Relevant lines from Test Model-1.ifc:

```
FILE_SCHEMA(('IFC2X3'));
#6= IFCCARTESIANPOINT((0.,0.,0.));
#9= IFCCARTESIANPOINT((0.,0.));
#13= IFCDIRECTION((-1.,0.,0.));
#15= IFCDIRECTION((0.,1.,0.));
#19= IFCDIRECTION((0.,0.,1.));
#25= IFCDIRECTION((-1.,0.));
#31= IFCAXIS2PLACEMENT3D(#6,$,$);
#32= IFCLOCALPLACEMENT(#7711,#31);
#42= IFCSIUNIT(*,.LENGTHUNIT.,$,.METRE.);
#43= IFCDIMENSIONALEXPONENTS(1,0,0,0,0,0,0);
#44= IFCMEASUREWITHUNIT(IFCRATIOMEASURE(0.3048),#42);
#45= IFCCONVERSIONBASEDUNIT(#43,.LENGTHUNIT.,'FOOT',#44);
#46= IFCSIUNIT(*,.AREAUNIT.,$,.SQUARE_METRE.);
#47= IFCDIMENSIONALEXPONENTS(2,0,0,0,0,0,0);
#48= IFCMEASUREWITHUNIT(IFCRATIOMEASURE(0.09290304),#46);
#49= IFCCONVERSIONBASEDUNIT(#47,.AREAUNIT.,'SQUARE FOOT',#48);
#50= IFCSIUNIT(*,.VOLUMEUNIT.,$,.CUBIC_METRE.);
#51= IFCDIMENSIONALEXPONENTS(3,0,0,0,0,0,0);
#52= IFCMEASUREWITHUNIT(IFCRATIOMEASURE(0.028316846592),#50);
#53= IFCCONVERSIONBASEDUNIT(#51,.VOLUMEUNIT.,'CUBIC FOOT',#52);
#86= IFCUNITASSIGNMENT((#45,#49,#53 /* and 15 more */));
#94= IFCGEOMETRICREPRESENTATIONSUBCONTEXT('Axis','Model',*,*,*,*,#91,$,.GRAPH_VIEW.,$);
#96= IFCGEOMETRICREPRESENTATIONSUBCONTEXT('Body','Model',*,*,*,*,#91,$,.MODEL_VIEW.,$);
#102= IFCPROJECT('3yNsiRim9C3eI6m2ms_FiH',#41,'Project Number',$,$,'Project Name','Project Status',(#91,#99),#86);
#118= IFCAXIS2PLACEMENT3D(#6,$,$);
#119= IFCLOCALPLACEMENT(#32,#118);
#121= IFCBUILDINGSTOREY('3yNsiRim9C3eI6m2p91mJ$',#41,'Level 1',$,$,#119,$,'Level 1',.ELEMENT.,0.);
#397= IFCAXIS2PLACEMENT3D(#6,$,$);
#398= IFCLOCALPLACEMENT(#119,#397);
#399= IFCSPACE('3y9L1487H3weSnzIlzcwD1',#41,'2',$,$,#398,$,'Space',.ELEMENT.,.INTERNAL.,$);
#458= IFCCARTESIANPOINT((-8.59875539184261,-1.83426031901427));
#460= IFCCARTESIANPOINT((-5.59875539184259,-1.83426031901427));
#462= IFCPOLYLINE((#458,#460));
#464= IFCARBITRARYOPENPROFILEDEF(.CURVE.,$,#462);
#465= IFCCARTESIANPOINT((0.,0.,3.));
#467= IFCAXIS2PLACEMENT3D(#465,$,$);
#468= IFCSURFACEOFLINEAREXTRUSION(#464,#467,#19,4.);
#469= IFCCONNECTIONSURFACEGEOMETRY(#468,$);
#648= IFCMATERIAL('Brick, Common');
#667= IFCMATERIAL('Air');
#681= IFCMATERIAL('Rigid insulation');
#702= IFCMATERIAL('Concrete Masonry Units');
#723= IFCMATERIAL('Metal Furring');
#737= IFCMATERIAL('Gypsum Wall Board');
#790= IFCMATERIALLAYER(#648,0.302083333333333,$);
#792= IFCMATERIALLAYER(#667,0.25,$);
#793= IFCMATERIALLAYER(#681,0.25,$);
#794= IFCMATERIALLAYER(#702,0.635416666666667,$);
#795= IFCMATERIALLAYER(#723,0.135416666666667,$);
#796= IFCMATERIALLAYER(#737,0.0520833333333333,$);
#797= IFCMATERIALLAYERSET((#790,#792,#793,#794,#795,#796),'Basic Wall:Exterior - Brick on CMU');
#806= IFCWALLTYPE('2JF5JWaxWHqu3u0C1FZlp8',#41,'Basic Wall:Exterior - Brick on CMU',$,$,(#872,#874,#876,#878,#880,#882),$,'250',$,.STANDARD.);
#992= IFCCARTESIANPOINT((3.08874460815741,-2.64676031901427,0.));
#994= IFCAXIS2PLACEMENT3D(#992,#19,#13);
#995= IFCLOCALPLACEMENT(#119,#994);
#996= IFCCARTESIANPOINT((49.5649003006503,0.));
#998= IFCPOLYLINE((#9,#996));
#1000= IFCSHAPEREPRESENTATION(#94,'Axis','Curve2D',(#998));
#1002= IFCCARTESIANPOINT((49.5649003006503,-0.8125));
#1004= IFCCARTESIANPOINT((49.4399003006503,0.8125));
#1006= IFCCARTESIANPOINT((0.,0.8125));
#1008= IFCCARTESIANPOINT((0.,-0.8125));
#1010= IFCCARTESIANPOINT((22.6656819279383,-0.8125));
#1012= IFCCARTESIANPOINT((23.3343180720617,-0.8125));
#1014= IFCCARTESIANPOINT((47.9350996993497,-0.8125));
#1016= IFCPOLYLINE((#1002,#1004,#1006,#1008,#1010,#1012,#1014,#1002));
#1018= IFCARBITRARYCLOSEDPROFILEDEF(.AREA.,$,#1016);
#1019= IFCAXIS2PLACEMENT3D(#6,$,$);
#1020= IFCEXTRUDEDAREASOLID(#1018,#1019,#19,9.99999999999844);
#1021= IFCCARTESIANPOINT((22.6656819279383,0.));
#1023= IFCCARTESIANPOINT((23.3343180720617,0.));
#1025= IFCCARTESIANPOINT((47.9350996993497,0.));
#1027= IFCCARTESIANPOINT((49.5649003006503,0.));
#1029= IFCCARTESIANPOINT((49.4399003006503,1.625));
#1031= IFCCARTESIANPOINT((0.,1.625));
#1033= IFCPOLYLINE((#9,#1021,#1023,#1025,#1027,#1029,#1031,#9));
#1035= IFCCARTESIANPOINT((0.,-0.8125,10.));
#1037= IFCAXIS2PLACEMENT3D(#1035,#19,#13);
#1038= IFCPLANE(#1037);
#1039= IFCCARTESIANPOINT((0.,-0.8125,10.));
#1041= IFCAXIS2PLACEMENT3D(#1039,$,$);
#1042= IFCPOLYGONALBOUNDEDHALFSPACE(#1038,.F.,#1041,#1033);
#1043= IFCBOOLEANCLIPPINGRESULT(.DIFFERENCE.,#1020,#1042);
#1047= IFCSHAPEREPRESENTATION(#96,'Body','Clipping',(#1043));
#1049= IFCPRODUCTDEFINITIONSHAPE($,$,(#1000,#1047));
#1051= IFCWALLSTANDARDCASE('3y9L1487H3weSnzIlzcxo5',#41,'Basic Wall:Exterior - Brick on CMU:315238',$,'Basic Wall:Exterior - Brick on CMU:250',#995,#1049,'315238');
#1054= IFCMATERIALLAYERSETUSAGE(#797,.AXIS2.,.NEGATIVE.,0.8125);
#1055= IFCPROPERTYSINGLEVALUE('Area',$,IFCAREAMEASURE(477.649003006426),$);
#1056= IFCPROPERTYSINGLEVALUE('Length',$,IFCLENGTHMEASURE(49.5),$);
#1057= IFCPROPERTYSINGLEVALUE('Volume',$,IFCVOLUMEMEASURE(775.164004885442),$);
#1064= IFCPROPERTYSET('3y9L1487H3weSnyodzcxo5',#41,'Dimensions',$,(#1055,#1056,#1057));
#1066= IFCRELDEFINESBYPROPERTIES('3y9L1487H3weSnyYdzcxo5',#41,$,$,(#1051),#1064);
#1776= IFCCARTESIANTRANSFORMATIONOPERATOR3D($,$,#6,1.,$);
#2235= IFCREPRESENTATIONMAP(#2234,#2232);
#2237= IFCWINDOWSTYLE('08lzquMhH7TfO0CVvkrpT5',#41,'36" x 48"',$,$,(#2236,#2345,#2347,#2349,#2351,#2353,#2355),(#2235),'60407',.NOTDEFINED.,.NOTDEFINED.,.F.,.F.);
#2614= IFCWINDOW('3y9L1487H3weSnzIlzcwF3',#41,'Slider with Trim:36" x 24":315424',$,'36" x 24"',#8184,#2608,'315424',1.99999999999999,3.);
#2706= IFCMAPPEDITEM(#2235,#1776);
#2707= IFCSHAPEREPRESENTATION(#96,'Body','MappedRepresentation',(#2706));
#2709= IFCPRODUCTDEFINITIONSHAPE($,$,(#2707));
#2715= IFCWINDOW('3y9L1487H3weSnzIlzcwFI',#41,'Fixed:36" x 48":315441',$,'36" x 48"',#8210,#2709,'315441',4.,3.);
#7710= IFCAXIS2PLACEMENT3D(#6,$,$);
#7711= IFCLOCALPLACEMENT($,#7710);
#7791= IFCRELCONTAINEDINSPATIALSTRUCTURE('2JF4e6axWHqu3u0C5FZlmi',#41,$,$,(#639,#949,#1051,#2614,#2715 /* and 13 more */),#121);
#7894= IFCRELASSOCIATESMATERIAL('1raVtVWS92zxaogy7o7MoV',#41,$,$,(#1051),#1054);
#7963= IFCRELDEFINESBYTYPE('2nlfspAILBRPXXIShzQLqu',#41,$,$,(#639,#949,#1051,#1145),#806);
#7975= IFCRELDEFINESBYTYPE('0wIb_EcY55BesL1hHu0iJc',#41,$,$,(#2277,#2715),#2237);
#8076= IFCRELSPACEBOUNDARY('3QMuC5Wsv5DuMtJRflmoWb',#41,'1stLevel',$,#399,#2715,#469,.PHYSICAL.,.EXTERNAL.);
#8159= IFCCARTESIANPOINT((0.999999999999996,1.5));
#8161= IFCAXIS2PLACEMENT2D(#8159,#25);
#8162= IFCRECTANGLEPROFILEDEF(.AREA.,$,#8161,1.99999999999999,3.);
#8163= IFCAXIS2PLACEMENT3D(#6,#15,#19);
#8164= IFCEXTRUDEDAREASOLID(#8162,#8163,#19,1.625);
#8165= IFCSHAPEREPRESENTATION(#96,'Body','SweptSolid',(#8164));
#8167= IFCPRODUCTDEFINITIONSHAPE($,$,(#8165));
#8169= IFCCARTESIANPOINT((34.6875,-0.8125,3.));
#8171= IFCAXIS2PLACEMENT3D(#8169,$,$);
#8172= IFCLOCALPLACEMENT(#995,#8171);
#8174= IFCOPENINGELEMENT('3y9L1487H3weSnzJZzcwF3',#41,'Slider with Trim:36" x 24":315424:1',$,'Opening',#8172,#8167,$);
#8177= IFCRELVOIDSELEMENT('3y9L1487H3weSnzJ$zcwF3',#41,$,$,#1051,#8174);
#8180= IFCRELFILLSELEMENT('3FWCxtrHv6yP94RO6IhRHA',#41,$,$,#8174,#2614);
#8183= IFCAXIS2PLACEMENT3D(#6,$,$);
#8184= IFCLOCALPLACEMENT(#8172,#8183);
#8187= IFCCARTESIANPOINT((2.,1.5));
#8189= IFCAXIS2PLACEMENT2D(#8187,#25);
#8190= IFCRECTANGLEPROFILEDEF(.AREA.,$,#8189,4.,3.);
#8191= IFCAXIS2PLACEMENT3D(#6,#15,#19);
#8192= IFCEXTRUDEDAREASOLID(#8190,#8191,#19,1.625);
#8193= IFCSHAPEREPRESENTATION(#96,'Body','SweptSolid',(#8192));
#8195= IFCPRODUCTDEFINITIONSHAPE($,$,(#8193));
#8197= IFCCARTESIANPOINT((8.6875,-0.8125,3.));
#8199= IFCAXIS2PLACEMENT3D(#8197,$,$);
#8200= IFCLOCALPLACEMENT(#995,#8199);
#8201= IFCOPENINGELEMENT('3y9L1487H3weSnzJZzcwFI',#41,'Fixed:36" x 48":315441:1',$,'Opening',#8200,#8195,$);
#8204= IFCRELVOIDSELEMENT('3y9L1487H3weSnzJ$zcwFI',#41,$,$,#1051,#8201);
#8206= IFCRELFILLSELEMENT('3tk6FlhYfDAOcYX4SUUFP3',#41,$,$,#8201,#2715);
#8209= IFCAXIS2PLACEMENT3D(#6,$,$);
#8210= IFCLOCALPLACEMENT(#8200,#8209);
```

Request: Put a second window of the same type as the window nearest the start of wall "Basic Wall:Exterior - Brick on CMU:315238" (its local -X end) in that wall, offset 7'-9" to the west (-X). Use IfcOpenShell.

```python
import numpy as np
import ifcopenshell
import ifcopenshell.api.feature
import ifcopenshell.api.geometry
import ifcopenshell.api.pset
import ifcopenshell.api.root
import ifcopenshell.geom
import ifcopenshell.util.element
import ifcopenshell.util.placement
import ifcopenshell.util.shape
import ifcopenshell.util.unit

model = ifcopenshell.open("Test Model-1.ifc")
unit_scale = ifcopenshell.util.unit.calculate_unit_scale(model)
area_scale = ifcopenshell.util.unit.calculate_unit_scale(model, "AREAUNIT")
volume_scale = ifcopenshell.util.unit.calculate_unit_scale(model, "VOLUMEUNIT")
settings = ifcopenshell.geom.settings()


def volume(element):
    """Net volume in cubic metres, openings subtracted."""
    shape = ifcopenshell.geom.create_shape(settings, element)
    return ifcopenshell.util.shape.get_volume(shape.geometry)


def reuse_history(source, copy):
    """copy_class also copies each property set's owner history, people and application; keep the originals."""
    for rel in copy.IsDefinedBy:
        if rel.is_a("IfcRelDefinesByProperties") and (history := rel.RelatingPropertyDefinition.OwnerHistory):
            rel.RelatingPropertyDefinition.OwnerHistory = source.OwnerHistory
            ifcopenshell.util.element.remove_deep2(model, history)


window = model.by_guid("3y9L1487H3weSnzIlzcwFI")
opening = window.FillsVoids[0].RelatingOpeningElement
wall = opening.VoidsElements[0].RelatingBuildingElement
before = volume(wall)
shift = ifcopenshell.util.placement.get_local_placement(wall.ObjectPlacement)[:3, 0] * 93 * 0.0254 / unit_scale

# copy_class copies the void relationship, type, container and properties, but no geometry.
new_opening = ifcopenshell.api.root.copy_class(model, product=opening)
new_opening.Representation = ifcopenshell.util.element.copy_deep(
    model, opening.Representation, exclude=["IfcGeometricRepresentationContext", "IfcRepresentationMap"]
)
new_opening.Name = 'Fixed:36" x 48"'
new_window = ifcopenshell.api.root.copy_class(model, product=window)
new_window.Representation = ifcopenshell.util.element.copy_deep(
    model, window.Representation, exclude=["IfcGeometricRepresentationContext", "IfcRepresentationMap"]
)
new_window.Name = 'Fixed:36" x 48"'
new_window.Tag = None
reuse_history(window, new_window)
fills = ifcopenshell.api.feature.add_filling(model, opening=new_opening, element=new_window)
fills.OwnerHistory = new_window.OwnerHistory  # required in IFC2X3

for old, new in ((opening, new_opening), (window, new_window)):
    matrix = ifcopenshell.util.placement.get_local_placement(old.ObjectPlacement)
    matrix[:3, 3] += shift
    ifcopenshell.api.geometry.edit_object_placement(model, product=new, matrix=matrix, is_si=False)

# The copied space boundaries still share their surfaces with the original.
for rel in new_window.ProvidesBoundaries:
    if rel.ConnectionGeometry:
        rel.ConnectionGeometry = ifcopenshell.util.element.copy_deep(model, rel.ConnectionGeometry)

# Space boundary surfaces are stored in each space's coordinates; move them too.
for rel in new_window.ProvidesBoundaries:
    if not rel.ConnectionGeometry:
        continue
    surface = rel.ConnectionGeometry.SurfaceOnRelatingElement
    space_matrix = ifcopenshell.util.placement.get_local_placement(rel.RelatingSpace.ObjectPlacement)
    point = np.array(surface.Position.Location.Coordinates) + space_matrix[:3, :3].T @ shift
    surface.Position = model.createIfcAxis2Placement3D(
        model.createIfcCartesianPoint(point.tolist()), surface.Position.Axis, surface.Position.RefDirection
    )

after = volume(wall)
thickness = 0.4953  # wall thickness in metres

# Update the wall's stored quantities.
pset = model.by_id(ifcopenshell.util.element.get_pset(wall, "Dimensions", should_inherit=False)["id"])
ifcopenshell.api.pset.edit_pset(model, pset=pset, properties={
    "Area": model.create_entity("IfcAreaMeasure", after / thickness / area_scale),
    "Volume": model.create_entity("IfcVolumeMeasure", after / volume_scale),
})

print(f"wall volume {before:.3f} -> {after:.3f} m3")

model.write("Test Model-1-out.ifc")
```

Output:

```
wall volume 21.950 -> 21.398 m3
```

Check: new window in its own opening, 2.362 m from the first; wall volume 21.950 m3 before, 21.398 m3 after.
